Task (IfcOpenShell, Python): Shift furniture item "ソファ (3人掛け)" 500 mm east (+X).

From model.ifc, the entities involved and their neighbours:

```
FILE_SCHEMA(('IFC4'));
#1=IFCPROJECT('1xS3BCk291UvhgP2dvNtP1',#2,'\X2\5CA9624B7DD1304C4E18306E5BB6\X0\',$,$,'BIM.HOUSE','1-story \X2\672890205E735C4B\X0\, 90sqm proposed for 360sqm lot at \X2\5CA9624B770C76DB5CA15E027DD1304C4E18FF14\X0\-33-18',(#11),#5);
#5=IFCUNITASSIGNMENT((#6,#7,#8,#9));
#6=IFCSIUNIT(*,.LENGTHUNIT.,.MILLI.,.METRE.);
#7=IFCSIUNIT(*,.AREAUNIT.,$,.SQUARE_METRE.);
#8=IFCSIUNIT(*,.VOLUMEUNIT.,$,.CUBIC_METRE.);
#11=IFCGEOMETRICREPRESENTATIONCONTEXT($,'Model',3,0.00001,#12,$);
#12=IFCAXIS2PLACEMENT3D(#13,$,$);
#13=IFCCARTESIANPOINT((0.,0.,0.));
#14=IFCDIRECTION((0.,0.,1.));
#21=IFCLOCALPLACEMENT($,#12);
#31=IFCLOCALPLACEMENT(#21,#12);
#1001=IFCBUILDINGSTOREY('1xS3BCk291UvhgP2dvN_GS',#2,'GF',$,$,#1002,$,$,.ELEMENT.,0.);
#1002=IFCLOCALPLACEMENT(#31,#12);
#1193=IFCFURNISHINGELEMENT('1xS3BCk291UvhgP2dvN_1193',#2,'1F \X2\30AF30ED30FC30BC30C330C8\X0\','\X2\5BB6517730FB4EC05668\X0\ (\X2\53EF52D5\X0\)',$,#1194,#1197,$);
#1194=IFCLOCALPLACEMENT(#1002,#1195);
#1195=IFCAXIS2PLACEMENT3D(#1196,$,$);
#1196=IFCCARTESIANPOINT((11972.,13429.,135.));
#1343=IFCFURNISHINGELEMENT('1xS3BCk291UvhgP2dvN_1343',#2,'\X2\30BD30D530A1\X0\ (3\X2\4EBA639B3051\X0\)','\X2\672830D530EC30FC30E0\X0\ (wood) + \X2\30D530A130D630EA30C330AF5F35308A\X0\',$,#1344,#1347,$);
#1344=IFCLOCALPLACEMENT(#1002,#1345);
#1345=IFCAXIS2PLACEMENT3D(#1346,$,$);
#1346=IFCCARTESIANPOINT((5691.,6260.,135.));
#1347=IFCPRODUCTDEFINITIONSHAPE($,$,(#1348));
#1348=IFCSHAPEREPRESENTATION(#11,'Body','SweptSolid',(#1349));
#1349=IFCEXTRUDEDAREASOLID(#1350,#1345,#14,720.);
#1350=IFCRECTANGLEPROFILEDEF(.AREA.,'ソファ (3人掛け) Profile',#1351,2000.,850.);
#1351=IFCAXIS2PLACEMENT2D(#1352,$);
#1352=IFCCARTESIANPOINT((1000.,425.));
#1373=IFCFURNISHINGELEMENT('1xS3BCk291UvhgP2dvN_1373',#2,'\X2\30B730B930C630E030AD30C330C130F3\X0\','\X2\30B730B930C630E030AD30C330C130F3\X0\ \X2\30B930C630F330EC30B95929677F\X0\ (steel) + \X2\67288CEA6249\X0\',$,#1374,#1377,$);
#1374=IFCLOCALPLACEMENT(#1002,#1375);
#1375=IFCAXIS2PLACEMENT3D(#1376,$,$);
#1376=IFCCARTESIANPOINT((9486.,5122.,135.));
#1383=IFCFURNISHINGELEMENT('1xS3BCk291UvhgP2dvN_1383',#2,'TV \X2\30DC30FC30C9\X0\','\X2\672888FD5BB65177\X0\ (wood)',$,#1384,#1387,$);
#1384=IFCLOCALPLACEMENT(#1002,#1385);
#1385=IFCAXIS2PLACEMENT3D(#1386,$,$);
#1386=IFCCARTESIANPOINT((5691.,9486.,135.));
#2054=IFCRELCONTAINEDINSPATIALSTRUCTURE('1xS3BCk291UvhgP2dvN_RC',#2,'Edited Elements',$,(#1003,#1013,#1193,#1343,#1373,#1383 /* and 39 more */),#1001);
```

```python
import ifcopenshell
import ifcopenshell.api.geometry
import ifcopenshell.util.placement
import ifcopenshell.util.unit

model = ifcopenshell.open("model.ifc")
unit_scale = ifcopenshell.util.unit.calculate_unit_scale(model)

item = model.by_guid("1xS3BCk291UvhgP2dvN_1343")
matrix = ifcopenshell.util.placement.get_local_placement(item.ObjectPlacement)
matrix[0, 3] += 0.5 / unit_scale
ifcopenshell.api.geometry.edit_object_placement(model, product=item, matrix=matrix, is_si=False)

print(ifcopenshell.util.placement.get_local_placement(item.ObjectPlacement).round(3) + 0.0)

model.write("model_v2.ifc")
```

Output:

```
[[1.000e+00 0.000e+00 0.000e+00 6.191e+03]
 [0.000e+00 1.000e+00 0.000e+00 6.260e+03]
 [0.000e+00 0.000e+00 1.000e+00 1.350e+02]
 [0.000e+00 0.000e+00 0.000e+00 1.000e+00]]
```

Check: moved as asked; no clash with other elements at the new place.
